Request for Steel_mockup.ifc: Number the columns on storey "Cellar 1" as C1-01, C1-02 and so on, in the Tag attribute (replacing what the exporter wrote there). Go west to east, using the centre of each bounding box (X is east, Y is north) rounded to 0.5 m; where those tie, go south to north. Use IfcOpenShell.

First a look at what the model holds.

```python
import ifcopenshell
import ifcopenshell.util.element
import ifcopenshell.util.placement

model = ifcopenshell.open("Steel_mockup.ifc")
print(model.schema)
storey = next(s for s in model.by_type("IfcBuildingStorey") if s.Name == "Cellar 1")
columns = [e for e in ifcopenshell.util.element.get_decomposition(storey) if e.is_a("IfcColumn")]
for e in sorted(columns, key=lambda e: e.id()):
    origin = ifcopenshell.util.placement.get_local_placement(e.ObjectPlacement)[:3, 3]
    print(e.id(), e.Tag, e.Name, origin.round(2) + 0.0, sep=" | ")
```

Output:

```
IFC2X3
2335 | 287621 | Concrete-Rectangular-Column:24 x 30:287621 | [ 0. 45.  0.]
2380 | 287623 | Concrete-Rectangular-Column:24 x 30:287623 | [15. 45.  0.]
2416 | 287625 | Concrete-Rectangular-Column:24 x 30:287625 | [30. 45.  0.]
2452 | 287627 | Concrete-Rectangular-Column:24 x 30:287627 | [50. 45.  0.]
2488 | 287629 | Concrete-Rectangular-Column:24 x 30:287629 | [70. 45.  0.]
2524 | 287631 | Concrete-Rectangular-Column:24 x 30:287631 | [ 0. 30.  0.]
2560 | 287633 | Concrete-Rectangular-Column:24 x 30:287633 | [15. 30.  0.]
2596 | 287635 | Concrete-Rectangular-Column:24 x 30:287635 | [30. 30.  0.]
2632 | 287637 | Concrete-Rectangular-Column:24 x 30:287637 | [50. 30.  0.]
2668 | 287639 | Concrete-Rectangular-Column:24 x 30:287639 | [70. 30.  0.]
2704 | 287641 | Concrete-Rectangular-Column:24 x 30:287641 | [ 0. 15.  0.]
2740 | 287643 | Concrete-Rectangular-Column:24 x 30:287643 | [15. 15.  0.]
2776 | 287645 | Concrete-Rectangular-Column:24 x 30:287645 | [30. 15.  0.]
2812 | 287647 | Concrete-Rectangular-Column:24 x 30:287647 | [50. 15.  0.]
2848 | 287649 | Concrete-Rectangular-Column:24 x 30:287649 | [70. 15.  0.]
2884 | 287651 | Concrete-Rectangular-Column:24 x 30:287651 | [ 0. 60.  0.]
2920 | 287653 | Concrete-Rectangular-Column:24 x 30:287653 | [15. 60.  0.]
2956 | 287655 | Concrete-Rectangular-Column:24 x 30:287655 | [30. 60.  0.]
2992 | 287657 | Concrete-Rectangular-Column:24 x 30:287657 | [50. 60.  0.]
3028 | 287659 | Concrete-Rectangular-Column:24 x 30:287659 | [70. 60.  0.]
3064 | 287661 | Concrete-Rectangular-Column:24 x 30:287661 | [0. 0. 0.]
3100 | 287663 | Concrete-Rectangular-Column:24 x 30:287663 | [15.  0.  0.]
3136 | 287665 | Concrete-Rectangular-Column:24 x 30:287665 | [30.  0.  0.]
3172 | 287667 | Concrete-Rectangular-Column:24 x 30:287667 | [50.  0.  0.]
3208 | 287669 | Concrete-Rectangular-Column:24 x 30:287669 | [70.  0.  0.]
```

```python
import ifcopenshell
import ifcopenshell.geom
import ifcopenshell.util.element
import ifcopenshell.util.shape

model = ifcopenshell.open("Steel_mockup.ifc")
settings = ifcopenshell.geom.settings()
settings.set("use-world-coords", True)


def centre(element):
    shape = ifcopenshell.geom.create_shape(settings, element)
    return ifcopenshell.util.shape.get_bbox_centroid(shape.geometry)


storey = next(s for s in model.by_type("IfcBuildingStorey") if s.Name == "Cellar 1")
columns = [e for e in ifcopenshell.util.element.get_decomposition(storey) if e.is_a("IfcColumn")]

# Insertion points can sit at a corner or the storey origin, so sort by the geometry (in metres).
centres = {e: centre(e) for e in columns}
columns.sort(key=lambda e: (round(centres[e][0] / 0.5), centres[e][1]))

for i, e in enumerate(columns, start=1):
    number = f"C1-{i:02d}"
    e.Tag = number
    print(e.id(), number)

model.write("Steel_mockup_rev.ifc")
```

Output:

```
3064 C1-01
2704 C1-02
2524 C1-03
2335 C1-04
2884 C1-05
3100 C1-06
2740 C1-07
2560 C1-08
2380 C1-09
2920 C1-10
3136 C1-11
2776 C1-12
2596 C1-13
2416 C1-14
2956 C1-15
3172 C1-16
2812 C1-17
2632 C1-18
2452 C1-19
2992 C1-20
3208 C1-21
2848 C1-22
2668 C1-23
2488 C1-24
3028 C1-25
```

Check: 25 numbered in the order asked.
